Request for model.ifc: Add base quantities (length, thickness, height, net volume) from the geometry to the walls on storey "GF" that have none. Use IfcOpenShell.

First a look at what the model holds.

```python
import ifcopenshell
import ifcopenshell.util.element
import ifcopenshell.util.unit

model = ifcopenshell.open("model.ifc")
print(model.schema)
for unit_type in ("LENGTHUNIT", "AREAUNIT", "VOLUMEUNIT"):
    print(unit_type, ifcopenshell.util.unit.calculate_unit_scale(model, unit_type))
storey = next(s for s in model.by_type("IfcBuildingStorey") if s.Name == "GF")
walls = [e for e in ifcopenshell.util.element.get_decomposition(storey) if e.is_a("IfcWall")]
for e in sorted(walls, key=lambda e: e.id()):
    print(e.id(), e.is_a(), e.Name, list(ifcopenshell.util.element.get_psets(e, qtos_only=True)), sep=" | ")
```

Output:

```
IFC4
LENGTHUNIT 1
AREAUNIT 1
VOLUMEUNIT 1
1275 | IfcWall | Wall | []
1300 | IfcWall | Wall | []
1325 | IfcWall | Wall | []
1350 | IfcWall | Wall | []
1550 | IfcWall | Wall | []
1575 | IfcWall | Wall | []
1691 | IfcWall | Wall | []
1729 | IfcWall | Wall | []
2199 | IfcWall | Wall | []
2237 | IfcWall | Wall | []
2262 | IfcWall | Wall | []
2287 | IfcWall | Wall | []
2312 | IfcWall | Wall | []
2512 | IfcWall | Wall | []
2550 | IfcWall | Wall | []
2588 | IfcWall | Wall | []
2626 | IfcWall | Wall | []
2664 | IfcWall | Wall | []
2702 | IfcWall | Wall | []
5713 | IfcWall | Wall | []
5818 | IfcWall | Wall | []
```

```python
import ifcopenshell
import ifcopenshell.api.pset
import ifcopenshell.geom
import ifcopenshell.util.element
import ifcopenshell.util.shape
import ifcopenshell.util.unit

model = ifcopenshell.open("model.ifc")
unit_scale = ifcopenshell.util.unit.calculate_unit_scale(model)
volume_scale = ifcopenshell.util.unit.calculate_unit_scale(model, "VOLUMEUNIT")
settings = ifcopenshell.geom.settings()

storey = next(s for s in model.by_type("IfcBuildingStorey") if s.Name == "GF")
walls = [e for e in ifcopenshell.util.element.get_decomposition(storey) if e.is_a("IfcWall")]

for e in sorted(walls, key=lambda e: e.id()):
    if ifcopenshell.util.element.get_psets(e, qtos_only=True, should_inherit=False):
        continue
    # Geometry comes back in metres, in the element's own axes.
    shape = ifcopenshell.geom.create_shape(settings, e)
    values = {
        "Length": ifcopenshell.util.shape.get_x(shape.geometry) / unit_scale,
        "Width": ifcopenshell.util.shape.get_y(shape.geometry) / unit_scale,
        "Height": ifcopenshell.util.shape.get_z(shape.geometry) / unit_scale,
        "NetVolume": ifcopenshell.util.shape.get_volume(shape.geometry) / volume_scale,
    }
    qto = ifcopenshell.api.pset.add_qto(model, product=e, name="Qto_WallBaseQuantities")
    ifcopenshell.api.pset.edit_qto(model, qto=qto, properties=values)
    print(e.id(), {k: round(v, 3) for k, v in values.items()})

model.write("model_rev.ifc")
```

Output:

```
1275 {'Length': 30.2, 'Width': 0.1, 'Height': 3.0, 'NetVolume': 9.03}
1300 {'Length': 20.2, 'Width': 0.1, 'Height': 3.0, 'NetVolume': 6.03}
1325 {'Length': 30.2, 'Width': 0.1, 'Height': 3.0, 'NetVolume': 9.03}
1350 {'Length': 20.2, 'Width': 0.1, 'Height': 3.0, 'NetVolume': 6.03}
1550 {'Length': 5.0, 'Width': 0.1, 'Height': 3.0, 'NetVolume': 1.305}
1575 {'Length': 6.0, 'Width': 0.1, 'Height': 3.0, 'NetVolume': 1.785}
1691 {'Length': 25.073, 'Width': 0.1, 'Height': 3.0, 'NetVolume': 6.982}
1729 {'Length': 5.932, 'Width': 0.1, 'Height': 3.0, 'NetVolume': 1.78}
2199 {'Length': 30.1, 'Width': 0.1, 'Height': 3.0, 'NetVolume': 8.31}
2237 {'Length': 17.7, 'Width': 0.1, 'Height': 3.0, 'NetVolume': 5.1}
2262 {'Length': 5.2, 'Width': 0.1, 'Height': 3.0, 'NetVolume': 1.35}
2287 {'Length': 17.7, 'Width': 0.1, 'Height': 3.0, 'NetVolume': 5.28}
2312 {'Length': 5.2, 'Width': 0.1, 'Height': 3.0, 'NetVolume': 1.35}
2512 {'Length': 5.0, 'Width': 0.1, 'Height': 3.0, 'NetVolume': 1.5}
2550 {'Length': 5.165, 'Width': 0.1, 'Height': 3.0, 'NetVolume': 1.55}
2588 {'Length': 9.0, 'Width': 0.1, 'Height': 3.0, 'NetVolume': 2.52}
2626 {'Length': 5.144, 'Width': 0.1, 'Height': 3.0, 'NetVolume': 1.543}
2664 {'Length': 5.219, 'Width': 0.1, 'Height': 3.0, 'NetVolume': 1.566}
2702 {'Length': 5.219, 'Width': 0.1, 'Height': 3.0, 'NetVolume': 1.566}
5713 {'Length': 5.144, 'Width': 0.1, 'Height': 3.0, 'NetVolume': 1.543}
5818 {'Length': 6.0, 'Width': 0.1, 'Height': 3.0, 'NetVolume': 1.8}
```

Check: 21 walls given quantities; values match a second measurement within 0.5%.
